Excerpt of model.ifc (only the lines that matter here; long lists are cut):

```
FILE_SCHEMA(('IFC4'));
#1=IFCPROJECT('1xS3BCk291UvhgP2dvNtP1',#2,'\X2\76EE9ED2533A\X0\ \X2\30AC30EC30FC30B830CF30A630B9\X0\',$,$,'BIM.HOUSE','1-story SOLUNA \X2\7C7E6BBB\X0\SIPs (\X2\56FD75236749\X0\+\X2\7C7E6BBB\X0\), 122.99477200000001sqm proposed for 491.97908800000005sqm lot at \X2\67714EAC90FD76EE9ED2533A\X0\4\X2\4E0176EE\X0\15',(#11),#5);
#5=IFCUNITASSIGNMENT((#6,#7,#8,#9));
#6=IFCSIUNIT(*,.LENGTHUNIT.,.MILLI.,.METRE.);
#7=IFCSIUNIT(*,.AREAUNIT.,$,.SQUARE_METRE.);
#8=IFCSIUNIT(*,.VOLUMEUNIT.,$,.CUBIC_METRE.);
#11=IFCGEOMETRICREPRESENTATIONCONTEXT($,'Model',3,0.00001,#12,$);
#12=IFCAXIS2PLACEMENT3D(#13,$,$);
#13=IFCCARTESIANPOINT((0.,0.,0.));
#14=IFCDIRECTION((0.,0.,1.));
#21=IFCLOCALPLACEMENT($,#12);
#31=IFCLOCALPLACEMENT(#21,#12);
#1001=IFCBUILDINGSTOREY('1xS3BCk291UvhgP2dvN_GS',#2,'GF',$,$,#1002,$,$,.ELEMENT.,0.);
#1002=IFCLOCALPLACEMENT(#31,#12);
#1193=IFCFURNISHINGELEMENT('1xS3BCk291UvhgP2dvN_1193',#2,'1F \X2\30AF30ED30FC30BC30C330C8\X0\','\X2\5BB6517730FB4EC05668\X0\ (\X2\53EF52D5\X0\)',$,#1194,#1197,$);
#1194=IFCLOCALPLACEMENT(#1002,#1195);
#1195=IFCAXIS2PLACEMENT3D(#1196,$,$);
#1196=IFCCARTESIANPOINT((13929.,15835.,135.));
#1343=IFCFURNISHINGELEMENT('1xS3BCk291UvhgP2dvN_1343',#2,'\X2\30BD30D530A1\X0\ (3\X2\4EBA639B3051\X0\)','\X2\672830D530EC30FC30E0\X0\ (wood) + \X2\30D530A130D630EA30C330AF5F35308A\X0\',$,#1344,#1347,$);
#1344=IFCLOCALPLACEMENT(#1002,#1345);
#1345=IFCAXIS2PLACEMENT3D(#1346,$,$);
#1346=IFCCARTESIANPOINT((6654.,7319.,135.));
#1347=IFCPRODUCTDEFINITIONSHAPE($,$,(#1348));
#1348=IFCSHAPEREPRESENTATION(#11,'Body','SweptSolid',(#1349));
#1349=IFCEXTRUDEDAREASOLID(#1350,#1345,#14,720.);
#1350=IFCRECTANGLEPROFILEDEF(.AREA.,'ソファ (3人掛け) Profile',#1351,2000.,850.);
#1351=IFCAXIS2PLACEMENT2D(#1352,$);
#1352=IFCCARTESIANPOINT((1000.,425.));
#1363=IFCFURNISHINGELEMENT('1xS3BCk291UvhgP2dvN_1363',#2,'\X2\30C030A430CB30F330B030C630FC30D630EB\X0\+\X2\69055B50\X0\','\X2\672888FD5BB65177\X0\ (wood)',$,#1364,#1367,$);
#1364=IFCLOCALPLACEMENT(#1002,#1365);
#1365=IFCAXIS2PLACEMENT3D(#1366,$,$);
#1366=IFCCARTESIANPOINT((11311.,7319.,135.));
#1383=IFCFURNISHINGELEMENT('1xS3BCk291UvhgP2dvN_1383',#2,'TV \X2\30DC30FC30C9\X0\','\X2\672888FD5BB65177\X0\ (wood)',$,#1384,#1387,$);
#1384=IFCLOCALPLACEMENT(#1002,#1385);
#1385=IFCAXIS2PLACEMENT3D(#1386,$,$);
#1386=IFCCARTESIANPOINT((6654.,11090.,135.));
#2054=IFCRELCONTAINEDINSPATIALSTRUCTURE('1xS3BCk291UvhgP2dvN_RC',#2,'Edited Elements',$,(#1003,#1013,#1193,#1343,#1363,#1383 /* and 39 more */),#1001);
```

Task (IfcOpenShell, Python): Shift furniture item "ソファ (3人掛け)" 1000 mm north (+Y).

```python
import ifcopenshell
import ifcopenshell.api.geometry
import ifcopenshell.util.placement

model = ifcopenshell.open("model.ifc")

item = model.by_guid("1xS3BCk291UvhgP2dvN_1343")
matrix = ifcopenshell.util.placement.get_local_placement(item.ObjectPlacement)
matrix[1, 3] += 1000.0
ifcopenshell.api.geometry.edit_object_placement(model, product=item, matrix=matrix, is_si=False)

print(ifcopenshell.util.placement.get_local_placement(item.ObjectPlacement).round(3) + 0.0)

model.write("model_v2.ifc")
```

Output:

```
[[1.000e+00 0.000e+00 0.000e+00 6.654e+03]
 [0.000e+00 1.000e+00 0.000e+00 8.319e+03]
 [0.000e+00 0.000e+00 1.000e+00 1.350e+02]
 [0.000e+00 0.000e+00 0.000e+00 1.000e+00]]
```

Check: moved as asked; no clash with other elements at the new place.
